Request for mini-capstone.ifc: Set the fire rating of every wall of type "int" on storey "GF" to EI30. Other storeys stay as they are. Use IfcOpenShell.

First a look at what the model holds.

```python
import ifcopenshell
import ifcopenshell.util.element

model = ifcopenshell.open("mini-capstone.ifc")
print(model.schema)
storey = next(s for s in model.by_type("IfcBuildingStorey") if s.Name == "GF")
walls = [e for e in ifcopenshell.util.element.get_decomposition(storey) if e.is_a("IfcWall")]
seen = {}
for e in walls:
    element_type = ifcopenshell.util.element.get_type(e)
    key = (element_type.Name if element_type != e and element_type else None, ifcopenshell.util.element.get_pset(e, "Pset_WallCommon", "FireRating"))
    seen[key] = seen.get(key, 0) + 1
for (name, value), count in sorted(seen.items(), key=str):
    print(count, "x", name, "|", value)
```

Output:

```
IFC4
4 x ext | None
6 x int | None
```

```python
import ifcopenshell
import ifcopenshell.api.pset
import ifcopenshell.util.element

model = ifcopenshell.open("mini-capstone.ifc")

storey = next(s for s in model.by_type("IfcBuildingStorey") if s.Name == "GF")
walls = [e for e in ifcopenshell.util.element.get_decomposition(storey) if e.is_a("IfcWall")]

count = 0
for e in walls:
    element_type = ifcopenshell.util.element.get_type(e)
    if element_type in (None, e) or element_type.Name != "int":
        continue
    # add_pset returns the element's existing set when there is one.
    pset = ifcopenshell.api.pset.add_pset(model, product=e, name="Pset_WallCommon")
    ifcopenshell.api.pset.edit_pset(model, pset=pset, properties={"FireRating": "EI30"})
    count += 1

print(count, "walls updated")

model.write("mini-capstone_edited.ifc")
```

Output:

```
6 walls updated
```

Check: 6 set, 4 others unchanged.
